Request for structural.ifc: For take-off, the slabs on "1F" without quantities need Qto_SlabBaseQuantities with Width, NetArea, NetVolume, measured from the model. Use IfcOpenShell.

First a look at what the model holds.

```python
import ifcopenshell
import ifcopenshell.util.element
import ifcopenshell.util.unit

model = ifcopenshell.open("structural.ifc")
print(model.schema)
for unit_type in ("LENGTHUNIT", "AREAUNIT", "VOLUMEUNIT"):
    print(unit_type, ifcopenshell.util.unit.calculate_unit_scale(model, unit_type))
storey = next(s for s in model.by_type("IfcBuildingStorey") if s.Name == "1F")
slabs = [e for e in ifcopenshell.util.element.get_decomposition(storey) if e.is_a("IfcSlab")]
for e in sorted(slabs, key=lambda e: e.id()):
    print(e.id(), e.is_a(), e.Name, list(ifcopenshell.util.element.get_psets(e, qtos_only=True)), sep=" | ")
```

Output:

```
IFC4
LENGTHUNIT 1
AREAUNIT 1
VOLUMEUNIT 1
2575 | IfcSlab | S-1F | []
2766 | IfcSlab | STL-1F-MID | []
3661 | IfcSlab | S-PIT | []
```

```python
import ifcopenshell
import ifcopenshell.api.pset
import ifcopenshell.geom
import ifcopenshell.util.element
import ifcopenshell.util.shape
import ifcopenshell.util.unit

model = ifcopenshell.open("structural.ifc")
unit_scale = ifcopenshell.util.unit.calculate_unit_scale(model)
area_scale = ifcopenshell.util.unit.calculate_unit_scale(model, "AREAUNIT")
volume_scale = ifcopenshell.util.unit.calculate_unit_scale(model, "VOLUMEUNIT")
settings = ifcopenshell.geom.settings()

storey = next(s for s in model.by_type("IfcBuildingStorey") if s.Name == "1F")
slabs = [e for e in ifcopenshell.util.element.get_decomposition(storey) if e.is_a("IfcSlab")]

for e in sorted(slabs, key=lambda e: e.id()):
    if ifcopenshell.util.element.get_psets(e, qtos_only=True, should_inherit=False):
        continue
    # Geometry comes back in metres, in the element's own axes.
    shape = ifcopenshell.geom.create_shape(settings, e)
    values = {
        "Width": ifcopenshell.util.shape.get_z(shape.geometry) / unit_scale,
        "NetArea": ifcopenshell.util.shape.get_footprint_area(shape.geometry) / area_scale,
        "NetVolume": ifcopenshell.util.shape.get_volume(shape.geometry) / volume_scale,
    }
    qto = ifcopenshell.api.pset.add_qto(model, product=e, name="Qto_SlabBaseQuantities")
    ifcopenshell.api.pset.edit_qto(model, qto=qto, properties=values)
    print(e.id(), {k: round(v, 3) for k, v in values.items()})

model.write("structural_updated.ifc")
```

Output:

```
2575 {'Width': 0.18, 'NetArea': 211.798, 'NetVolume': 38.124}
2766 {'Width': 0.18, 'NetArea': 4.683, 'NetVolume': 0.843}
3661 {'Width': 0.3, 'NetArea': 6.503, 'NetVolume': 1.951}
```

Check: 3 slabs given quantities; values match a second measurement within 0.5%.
